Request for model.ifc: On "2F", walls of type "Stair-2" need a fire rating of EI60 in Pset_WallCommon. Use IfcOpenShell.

First a look at what the model holds.

```python
import ifcopenshell
import ifcopenshell.util.element

model = ifcopenshell.open("model.ifc")
print(model.schema)
storey = next(s for s in model.by_type("IfcBuildingStorey") if s.Name == "2F")
walls = [e for e in ifcopenshell.util.element.get_decomposition(storey) if e.is_a("IfcWall")]
seen = {}
for e in walls:
    element_type = ifcopenshell.util.element.get_type(e)
    key = (element_type.Name if element_type != e and element_type else None, ifcopenshell.util.element.get_pset(e, "Pset_WallCommon", "FireRating"))
    seen[key] = seen.get(key, 0) + 1
for (name, value), count in sorted(seen.items(), key=str):
    print(count, "x", name, "|", value)
```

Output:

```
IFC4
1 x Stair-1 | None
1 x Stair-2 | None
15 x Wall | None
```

```python
import ifcopenshell
import ifcopenshell.api.pset
import ifcopenshell.util.element

model = ifcopenshell.open("model.ifc")

storey = next(s for s in model.by_type("IfcBuildingStorey") if s.Name == "2F")
walls = [e for e in ifcopenshell.util.element.get_decomposition(storey) if e.is_a("IfcWall")]

count = 0
for e in walls:
    element_type = ifcopenshell.util.element.get_type(e)
    if element_type in (None, e) or element_type.Name != "Stair-2":
        continue
    # add_pset returns the element's existing set when there is one.
    pset = ifcopenshell.api.pset.add_pset(model, product=e, name="Pset_WallCommon")
    ifcopenshell.api.pset.edit_pset(model, pset=pset, properties={"FireRating": "EI60"})
    count += 1

print(count, "walls updated")

model.write("model_edited.ifc")
```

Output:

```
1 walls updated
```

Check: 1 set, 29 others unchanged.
